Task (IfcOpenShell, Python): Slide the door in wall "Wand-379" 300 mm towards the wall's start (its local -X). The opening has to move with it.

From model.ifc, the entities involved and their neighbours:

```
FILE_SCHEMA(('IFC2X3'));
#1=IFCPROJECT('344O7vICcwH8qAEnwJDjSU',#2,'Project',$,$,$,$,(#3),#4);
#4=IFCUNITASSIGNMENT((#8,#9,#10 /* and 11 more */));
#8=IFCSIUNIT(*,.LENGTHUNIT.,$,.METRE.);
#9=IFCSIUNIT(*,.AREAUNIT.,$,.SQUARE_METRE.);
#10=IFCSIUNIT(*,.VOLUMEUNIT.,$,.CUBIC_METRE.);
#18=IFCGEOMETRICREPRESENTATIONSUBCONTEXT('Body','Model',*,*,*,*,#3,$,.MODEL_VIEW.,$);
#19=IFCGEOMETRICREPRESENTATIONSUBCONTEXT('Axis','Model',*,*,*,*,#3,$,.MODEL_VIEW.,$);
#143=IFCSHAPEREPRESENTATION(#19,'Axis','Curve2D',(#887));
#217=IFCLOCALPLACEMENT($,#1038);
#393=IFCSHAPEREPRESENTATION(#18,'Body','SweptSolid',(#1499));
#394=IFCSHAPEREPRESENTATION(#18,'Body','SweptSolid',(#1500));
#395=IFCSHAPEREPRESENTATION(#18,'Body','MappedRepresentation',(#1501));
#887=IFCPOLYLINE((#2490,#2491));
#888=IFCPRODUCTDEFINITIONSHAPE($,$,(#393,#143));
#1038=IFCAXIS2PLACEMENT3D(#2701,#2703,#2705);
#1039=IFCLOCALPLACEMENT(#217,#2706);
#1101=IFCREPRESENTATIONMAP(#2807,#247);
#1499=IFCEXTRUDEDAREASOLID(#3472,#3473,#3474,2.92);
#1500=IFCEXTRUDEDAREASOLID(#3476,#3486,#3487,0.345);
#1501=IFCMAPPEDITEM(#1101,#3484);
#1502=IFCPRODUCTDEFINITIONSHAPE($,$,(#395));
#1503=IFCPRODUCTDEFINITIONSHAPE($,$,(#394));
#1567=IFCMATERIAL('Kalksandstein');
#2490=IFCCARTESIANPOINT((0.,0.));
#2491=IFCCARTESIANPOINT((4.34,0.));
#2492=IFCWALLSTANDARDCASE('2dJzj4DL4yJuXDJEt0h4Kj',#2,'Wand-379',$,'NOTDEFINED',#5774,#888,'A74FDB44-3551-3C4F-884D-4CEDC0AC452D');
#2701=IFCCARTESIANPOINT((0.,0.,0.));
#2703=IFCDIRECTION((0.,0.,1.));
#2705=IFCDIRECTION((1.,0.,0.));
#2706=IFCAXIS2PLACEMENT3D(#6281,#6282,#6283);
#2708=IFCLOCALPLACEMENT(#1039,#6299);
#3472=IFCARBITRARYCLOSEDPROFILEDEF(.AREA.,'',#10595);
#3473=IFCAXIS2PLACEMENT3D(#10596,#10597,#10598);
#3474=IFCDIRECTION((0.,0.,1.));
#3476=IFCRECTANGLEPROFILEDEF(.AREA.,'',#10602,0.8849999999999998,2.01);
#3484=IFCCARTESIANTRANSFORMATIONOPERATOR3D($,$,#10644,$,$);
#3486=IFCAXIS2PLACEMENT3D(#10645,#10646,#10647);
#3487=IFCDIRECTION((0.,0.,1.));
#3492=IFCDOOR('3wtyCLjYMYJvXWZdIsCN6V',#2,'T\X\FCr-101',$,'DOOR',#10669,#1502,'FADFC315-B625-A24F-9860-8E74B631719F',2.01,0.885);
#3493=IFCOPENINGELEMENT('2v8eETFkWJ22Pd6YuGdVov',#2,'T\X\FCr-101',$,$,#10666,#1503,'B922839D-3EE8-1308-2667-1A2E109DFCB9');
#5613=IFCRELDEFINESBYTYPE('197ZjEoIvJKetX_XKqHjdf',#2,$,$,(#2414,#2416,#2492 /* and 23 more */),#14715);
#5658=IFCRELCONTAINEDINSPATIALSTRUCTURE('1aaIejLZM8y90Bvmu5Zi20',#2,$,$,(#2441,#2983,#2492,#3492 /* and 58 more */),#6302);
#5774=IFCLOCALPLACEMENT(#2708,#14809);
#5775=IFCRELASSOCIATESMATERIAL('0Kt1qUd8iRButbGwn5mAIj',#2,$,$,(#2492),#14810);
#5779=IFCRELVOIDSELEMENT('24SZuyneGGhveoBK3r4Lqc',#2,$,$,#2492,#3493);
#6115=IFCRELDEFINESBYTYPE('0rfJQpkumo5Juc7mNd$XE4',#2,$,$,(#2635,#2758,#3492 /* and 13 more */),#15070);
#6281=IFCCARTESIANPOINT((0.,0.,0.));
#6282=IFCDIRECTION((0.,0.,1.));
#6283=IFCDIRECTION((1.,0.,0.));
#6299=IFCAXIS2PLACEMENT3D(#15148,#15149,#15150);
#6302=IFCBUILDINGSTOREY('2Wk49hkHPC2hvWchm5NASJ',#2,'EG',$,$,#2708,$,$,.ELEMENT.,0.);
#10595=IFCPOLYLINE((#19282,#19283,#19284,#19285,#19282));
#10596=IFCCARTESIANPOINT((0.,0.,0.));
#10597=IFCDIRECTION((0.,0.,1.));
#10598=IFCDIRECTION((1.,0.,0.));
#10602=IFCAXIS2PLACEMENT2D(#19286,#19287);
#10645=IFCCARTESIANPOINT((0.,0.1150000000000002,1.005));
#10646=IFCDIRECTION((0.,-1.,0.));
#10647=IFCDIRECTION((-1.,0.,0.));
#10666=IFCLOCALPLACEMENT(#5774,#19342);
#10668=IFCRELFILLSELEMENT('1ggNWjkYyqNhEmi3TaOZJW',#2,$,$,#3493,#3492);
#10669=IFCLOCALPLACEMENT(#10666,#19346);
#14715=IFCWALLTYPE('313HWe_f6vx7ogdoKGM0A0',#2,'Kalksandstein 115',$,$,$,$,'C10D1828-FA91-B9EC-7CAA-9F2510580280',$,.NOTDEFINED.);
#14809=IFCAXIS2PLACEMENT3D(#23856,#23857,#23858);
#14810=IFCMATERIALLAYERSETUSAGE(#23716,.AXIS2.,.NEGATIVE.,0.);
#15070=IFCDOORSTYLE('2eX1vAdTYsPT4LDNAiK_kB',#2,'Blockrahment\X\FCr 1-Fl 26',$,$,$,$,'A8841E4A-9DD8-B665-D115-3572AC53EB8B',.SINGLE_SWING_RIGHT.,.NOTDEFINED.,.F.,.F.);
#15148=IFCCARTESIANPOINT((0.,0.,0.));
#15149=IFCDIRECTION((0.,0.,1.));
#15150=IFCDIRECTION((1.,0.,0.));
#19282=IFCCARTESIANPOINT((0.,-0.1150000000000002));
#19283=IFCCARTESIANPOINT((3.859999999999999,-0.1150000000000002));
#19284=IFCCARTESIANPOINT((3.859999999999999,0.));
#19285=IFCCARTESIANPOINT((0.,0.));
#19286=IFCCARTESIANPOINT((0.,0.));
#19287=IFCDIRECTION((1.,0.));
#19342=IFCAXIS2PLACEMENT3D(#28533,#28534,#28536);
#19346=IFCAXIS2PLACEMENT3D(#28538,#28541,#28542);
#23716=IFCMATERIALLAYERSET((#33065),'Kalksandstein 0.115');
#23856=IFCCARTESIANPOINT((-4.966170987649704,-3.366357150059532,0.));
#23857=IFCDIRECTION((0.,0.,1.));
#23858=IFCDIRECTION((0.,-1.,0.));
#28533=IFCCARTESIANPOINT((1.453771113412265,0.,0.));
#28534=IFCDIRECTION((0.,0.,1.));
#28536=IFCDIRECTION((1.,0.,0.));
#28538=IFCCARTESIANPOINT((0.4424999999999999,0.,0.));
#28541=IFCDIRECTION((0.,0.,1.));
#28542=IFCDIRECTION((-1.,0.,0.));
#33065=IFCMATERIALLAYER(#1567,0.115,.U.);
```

```python
import ifcopenshell
import ifcopenshell.api.geometry
import ifcopenshell.util.placement
import ifcopenshell.util.unit

model = ifcopenshell.open("model.ifc")
unit_scale = ifcopenshell.util.unit.calculate_unit_scale(model)

door = model.by_guid("3wtyCLjYMYJvXWZdIsCN6V")
opening = door.FillsVoids[0].RelatingOpeningElement
wall = opening.VoidsElements[0].RelatingBuildingElement

wall_matrix = ifcopenshell.util.placement.get_local_placement(wall.ObjectPlacement)
shift = wall_matrix[:3, 0] * -0.3 / unit_scale
before = ifcopenshell.util.placement.get_local_placement(door.ObjectPlacement)[:3, 3].copy()

# The door is placed relative to its opening, so it follows when the opening moves.
matrix = ifcopenshell.util.placement.get_local_placement(opening.ObjectPlacement)
matrix[:3, 3] += shift
ifcopenshell.api.geometry.edit_object_placement(
    model, product=opening, matrix=matrix, is_si=False, should_transform_children=True
)

after = ifcopenshell.util.placement.get_local_placement(door.ObjectPlacement)[:3, 3]
print("door moved by", (after - before).round(3) + 0.0)

model.write("model_rev.ifc")
```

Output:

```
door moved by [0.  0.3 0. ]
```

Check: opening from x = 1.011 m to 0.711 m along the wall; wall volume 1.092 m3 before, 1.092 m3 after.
